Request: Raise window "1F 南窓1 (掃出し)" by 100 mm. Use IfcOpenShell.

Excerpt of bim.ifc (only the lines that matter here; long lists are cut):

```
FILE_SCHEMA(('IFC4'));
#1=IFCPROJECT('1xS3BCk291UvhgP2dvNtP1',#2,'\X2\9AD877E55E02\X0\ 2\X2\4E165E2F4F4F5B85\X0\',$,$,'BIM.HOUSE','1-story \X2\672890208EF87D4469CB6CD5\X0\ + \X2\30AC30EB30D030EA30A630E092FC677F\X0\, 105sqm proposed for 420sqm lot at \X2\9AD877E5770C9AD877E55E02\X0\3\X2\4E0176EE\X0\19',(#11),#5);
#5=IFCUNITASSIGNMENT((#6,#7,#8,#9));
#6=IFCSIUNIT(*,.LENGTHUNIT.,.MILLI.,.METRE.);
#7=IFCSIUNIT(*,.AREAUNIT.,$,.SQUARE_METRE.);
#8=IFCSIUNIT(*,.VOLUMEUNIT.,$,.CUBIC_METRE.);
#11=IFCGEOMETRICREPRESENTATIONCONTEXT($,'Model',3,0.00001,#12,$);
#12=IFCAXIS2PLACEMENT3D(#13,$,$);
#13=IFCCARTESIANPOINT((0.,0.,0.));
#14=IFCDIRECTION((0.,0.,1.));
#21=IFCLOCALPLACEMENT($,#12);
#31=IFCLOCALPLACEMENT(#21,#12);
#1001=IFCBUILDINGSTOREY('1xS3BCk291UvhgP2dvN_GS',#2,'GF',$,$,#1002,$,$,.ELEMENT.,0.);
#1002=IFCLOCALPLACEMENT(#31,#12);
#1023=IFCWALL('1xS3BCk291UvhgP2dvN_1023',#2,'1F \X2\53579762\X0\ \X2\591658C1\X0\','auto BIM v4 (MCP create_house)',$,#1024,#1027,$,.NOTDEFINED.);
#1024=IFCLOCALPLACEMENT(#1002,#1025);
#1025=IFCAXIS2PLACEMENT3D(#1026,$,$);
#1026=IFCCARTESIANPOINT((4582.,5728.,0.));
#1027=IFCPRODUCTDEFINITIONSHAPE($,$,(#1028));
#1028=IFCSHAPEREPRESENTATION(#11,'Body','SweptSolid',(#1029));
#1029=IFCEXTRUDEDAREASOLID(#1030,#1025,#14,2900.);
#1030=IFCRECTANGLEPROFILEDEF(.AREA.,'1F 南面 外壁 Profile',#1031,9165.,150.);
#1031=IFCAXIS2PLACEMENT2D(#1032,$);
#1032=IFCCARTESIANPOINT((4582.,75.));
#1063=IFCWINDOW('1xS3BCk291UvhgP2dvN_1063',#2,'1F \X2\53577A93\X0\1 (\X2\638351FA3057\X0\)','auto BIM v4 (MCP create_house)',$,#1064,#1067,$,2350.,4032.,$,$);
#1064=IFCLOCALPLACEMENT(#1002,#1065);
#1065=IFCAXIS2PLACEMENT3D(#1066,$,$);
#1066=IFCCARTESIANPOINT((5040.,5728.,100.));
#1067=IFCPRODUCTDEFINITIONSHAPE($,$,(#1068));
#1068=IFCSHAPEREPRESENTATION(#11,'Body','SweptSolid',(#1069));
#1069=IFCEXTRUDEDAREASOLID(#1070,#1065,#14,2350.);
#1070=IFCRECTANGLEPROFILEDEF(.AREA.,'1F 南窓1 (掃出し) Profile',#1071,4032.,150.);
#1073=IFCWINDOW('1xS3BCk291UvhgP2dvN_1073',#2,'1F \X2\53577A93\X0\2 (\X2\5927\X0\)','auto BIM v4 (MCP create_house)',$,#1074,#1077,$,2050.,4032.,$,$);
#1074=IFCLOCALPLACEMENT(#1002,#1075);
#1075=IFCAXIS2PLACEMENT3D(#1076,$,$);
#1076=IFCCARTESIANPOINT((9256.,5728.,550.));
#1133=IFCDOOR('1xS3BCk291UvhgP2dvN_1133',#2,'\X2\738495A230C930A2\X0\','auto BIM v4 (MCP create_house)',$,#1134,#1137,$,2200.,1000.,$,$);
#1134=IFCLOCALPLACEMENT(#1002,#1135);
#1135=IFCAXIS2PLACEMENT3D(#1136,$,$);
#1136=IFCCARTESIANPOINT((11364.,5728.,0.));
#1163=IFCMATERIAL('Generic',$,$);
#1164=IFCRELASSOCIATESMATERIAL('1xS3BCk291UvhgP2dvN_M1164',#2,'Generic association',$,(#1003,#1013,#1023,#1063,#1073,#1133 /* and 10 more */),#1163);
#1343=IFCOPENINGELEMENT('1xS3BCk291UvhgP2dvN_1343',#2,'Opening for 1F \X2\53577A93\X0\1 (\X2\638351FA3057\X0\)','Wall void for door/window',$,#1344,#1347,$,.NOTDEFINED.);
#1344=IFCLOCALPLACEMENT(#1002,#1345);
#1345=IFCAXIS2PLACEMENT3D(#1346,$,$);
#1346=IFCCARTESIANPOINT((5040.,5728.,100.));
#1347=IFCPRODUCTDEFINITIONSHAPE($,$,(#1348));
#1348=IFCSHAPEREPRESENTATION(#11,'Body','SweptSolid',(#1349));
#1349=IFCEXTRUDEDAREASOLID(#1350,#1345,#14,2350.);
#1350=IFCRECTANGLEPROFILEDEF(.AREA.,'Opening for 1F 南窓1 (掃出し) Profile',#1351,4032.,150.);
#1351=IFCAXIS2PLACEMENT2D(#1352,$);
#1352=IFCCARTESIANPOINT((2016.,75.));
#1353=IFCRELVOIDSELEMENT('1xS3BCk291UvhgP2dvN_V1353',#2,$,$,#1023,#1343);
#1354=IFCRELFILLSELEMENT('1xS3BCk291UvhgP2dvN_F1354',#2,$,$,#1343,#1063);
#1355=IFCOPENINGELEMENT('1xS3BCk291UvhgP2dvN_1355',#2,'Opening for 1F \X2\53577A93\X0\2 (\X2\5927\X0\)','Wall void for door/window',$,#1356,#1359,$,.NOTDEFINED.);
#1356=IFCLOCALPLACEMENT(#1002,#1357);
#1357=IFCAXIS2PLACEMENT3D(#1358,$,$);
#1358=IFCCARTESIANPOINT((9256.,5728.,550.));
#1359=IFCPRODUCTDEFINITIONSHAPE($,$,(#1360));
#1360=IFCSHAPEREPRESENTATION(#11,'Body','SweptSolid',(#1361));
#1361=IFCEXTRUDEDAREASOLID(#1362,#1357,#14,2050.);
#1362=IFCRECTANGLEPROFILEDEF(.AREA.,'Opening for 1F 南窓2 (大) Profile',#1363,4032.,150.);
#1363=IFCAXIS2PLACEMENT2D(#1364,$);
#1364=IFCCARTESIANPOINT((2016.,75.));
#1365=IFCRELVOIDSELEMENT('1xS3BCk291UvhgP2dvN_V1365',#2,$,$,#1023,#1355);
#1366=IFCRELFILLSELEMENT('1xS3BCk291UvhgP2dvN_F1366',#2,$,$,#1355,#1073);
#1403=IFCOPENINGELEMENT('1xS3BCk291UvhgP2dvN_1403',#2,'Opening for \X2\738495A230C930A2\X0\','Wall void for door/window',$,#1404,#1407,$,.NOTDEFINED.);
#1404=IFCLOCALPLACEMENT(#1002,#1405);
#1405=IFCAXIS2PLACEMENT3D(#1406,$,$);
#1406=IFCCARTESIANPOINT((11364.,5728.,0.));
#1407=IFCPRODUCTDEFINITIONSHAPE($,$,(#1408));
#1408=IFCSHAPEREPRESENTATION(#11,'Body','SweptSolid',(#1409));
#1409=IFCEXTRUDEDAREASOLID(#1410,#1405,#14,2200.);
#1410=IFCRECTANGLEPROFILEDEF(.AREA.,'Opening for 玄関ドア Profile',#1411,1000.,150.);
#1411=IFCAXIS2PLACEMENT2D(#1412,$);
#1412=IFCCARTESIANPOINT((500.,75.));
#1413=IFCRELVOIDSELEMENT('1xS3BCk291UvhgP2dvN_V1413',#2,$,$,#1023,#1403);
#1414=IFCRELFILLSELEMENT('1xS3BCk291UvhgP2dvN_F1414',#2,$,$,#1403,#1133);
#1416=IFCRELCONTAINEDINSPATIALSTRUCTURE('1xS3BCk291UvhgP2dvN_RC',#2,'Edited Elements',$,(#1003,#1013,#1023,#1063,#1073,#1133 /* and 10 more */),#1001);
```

```python
import numpy as np
import ifcopenshell
import ifcopenshell.api.geometry
import ifcopenshell.util.placement
import ifcopenshell.util.unit

model = ifcopenshell.open("bim.ifc")
unit_scale = ifcopenshell.util.unit.calculate_unit_scale(model)

window = model.by_guid("1xS3BCk291UvhgP2dvN_1063")
opening = window.FillsVoids[0].RelatingOpeningElement
dz = 100.0

shift = np.array([0.0, 0.0, dz])
# The window is not placed relative to its opening, so move both.
for product in (opening, window):
    matrix = ifcopenshell.util.placement.get_local_placement(product.ObjectPlacement)
    matrix[:3, 3] += shift
    ifcopenshell.api.geometry.edit_object_placement(model, product=product, matrix=matrix, is_si=False)

print(f"moved by {dz * unit_scale:+.3f} m")

model.write("bim-out.ifc")
```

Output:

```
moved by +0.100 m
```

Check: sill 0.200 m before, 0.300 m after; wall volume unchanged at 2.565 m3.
